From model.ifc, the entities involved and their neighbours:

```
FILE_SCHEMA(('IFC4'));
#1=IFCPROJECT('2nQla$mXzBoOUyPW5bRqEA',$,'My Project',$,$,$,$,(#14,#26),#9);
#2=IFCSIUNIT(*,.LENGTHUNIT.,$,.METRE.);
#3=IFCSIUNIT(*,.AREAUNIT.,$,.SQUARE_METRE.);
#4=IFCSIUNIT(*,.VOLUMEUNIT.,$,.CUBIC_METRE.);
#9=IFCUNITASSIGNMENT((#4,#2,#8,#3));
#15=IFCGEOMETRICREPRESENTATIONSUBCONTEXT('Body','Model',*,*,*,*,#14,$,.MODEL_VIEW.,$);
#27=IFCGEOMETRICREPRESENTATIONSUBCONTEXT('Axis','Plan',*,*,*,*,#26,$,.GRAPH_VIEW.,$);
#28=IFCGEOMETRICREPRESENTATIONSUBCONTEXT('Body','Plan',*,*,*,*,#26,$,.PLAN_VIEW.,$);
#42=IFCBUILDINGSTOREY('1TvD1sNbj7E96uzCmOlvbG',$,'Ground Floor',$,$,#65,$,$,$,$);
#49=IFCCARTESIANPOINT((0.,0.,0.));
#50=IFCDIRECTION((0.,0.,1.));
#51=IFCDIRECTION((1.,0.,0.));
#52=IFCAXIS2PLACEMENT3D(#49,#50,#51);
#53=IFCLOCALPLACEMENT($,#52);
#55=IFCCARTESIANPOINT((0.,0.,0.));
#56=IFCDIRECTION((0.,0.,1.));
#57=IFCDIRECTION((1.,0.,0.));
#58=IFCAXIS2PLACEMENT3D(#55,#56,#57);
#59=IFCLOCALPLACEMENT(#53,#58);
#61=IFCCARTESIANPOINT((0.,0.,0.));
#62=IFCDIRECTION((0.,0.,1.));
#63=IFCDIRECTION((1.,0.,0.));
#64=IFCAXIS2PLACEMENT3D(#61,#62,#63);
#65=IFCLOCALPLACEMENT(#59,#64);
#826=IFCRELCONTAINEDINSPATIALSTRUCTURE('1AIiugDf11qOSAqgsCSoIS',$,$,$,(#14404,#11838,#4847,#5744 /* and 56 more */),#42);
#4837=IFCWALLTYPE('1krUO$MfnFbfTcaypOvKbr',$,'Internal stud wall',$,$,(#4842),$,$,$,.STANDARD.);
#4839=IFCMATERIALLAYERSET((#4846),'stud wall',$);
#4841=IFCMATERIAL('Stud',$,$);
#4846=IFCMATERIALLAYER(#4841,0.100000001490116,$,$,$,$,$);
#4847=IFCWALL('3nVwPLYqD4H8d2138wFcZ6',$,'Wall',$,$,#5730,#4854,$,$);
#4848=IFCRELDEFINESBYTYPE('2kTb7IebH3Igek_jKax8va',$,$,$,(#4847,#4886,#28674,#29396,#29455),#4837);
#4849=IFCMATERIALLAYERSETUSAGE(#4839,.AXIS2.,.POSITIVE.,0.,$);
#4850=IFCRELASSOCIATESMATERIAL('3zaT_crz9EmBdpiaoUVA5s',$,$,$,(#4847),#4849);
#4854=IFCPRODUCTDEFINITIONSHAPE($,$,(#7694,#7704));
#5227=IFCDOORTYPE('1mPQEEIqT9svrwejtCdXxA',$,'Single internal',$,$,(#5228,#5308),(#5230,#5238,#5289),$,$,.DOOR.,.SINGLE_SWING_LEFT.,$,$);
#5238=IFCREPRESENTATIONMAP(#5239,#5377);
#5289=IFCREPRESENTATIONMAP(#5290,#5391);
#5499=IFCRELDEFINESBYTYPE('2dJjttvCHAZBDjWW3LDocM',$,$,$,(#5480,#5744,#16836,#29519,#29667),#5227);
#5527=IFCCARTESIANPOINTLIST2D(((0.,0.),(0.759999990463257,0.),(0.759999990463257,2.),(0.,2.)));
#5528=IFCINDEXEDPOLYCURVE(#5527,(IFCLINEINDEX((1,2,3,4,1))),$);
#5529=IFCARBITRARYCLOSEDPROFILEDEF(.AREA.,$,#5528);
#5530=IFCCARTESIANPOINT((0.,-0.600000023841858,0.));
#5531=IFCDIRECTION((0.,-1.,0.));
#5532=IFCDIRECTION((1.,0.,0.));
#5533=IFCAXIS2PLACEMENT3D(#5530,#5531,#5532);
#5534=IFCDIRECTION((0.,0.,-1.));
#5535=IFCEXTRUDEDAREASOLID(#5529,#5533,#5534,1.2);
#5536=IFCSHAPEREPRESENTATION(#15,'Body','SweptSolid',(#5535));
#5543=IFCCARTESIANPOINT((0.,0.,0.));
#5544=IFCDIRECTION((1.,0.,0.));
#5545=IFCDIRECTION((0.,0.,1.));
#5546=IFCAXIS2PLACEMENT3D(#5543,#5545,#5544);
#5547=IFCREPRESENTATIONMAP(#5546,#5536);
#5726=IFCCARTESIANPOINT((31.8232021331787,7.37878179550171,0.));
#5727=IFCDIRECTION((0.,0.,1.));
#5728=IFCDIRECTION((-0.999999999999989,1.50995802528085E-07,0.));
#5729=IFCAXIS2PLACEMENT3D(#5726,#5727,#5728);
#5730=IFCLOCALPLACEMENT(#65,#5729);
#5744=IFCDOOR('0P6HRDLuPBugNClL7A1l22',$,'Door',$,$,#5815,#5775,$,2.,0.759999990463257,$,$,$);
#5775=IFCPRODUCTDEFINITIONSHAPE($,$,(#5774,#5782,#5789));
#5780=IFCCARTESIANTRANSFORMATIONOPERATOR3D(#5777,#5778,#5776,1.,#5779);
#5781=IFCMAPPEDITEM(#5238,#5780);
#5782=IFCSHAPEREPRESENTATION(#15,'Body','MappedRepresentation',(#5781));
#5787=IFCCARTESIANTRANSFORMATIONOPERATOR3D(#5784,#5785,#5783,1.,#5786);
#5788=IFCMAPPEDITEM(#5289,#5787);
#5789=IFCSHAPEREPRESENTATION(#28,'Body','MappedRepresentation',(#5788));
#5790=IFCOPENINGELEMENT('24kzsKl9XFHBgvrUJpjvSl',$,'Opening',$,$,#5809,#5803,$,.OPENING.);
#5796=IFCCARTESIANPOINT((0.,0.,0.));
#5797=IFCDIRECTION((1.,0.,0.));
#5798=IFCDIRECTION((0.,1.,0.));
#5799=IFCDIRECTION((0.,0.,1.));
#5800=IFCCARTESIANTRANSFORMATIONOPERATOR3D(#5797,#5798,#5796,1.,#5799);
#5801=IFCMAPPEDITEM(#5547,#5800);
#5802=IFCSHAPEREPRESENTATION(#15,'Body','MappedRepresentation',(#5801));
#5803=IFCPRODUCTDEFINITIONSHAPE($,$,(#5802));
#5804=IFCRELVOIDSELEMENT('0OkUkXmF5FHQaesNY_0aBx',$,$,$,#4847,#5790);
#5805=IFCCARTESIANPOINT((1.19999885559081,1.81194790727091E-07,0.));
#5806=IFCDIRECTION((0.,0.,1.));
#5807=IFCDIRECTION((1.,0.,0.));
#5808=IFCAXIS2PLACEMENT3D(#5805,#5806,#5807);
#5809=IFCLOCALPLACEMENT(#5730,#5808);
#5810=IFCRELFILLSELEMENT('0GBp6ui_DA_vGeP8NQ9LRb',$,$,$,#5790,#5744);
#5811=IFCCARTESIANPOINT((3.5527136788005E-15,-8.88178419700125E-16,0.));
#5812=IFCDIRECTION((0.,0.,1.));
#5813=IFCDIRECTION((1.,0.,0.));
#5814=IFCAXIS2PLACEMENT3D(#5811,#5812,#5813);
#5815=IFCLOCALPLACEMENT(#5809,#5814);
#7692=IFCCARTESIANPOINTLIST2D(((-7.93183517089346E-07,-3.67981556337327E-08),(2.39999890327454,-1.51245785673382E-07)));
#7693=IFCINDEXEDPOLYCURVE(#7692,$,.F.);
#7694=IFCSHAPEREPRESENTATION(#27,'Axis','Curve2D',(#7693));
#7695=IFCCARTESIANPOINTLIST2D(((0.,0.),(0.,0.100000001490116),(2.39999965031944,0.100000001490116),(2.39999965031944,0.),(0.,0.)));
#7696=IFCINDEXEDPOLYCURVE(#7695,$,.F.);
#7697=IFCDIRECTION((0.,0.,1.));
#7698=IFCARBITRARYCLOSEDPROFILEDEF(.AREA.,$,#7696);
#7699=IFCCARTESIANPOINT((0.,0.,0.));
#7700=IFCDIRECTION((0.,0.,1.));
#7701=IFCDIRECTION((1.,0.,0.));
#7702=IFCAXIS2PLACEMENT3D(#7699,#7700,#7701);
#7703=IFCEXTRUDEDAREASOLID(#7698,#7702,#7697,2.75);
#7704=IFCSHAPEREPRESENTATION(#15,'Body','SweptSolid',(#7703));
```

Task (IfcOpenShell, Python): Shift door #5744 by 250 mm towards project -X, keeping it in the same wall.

```python
import ifcopenshell
import ifcopenshell.api.geometry
import ifcopenshell.util.placement
import ifcopenshell.util.unit

model = ifcopenshell.open("model.ifc")
unit_scale = ifcopenshell.util.unit.calculate_unit_scale(model)

door = model.by_id(5744)
opening = door.FillsVoids[0].RelatingOpeningElement
wall = opening.VoidsElements[0].RelatingBuildingElement

wall_matrix = ifcopenshell.util.placement.get_local_placement(wall.ObjectPlacement)
shift = wall_matrix[:3, 0] * 0.25 / unit_scale
before = ifcopenshell.util.placement.get_local_placement(door.ObjectPlacement)[:3, 3].copy()

# The door is placed relative to its opening, so it follows when the opening moves.
matrix = ifcopenshell.util.placement.get_local_placement(opening.ObjectPlacement)
matrix[:3, 3] += shift
ifcopenshell.api.geometry.edit_object_placement(
    model, product=opening, matrix=matrix, is_si=False, should_transform_children=True
)

after = ifcopenshell.util.placement.get_local_placement(door.ObjectPlacement)[:3, 3]
print("door moved by", (after - before).round(3) + 0.0)

model.write("model_rev.ifc")
```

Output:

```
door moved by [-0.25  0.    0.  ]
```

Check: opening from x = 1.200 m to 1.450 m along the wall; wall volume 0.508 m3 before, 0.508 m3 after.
